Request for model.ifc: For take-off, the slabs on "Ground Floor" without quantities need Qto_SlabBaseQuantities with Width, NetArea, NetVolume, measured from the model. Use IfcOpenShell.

First a look at what the model holds.

```python
import ifcopenshell
import ifcopenshell.util.element
import ifcopenshell.util.unit

model = ifcopenshell.open("model.ifc")
print(model.schema)
for unit_type in ("LENGTHUNIT", "AREAUNIT", "VOLUMEUNIT"):
    print(unit_type, ifcopenshell.util.unit.calculate_unit_scale(model, unit_type))
storey = next(s for s in model.by_type("IfcBuildingStorey") if s.Name == "Ground Floor")
slabs = [e for e in ifcopenshell.util.element.get_decomposition(storey) if e.is_a("IfcSlab")]
for e in sorted(slabs, key=lambda e: e.id()):
    print(e.id(), e.is_a(), e.Name, list(ifcopenshell.util.element.get_psets(e, qtos_only=True)), sep=" | ")
```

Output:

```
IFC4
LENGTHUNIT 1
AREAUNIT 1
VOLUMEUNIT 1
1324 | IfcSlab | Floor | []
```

```python
import ifcopenshell
import ifcopenshell.api.pset
import ifcopenshell.geom
import ifcopenshell.util.element
import ifcopenshell.util.shape
import ifcopenshell.util.unit

model = ifcopenshell.open("model.ifc")
unit_scale = ifcopenshell.util.unit.calculate_unit_scale(model)
area_scale = ifcopenshell.util.unit.calculate_unit_scale(model, "AREAUNIT")
volume_scale = ifcopenshell.util.unit.calculate_unit_scale(model, "VOLUMEUNIT")
settings = ifcopenshell.geom.settings()

storey = next(s for s in model.by_type("IfcBuildingStorey") if s.Name == "Ground Floor")
slabs = [e for e in ifcopenshell.util.element.get_decomposition(storey) if e.is_a("IfcSlab")]

for e in sorted(slabs, key=lambda e: e.id()):
    if ifcopenshell.util.element.get_psets(e, qtos_only=True, should_inherit=False):
        continue
    # Geometry comes back in metres, in the element's own axes.
    shape = ifcopenshell.geom.create_shape(settings, e)
    values = {
        "Width": ifcopenshell.util.shape.get_z(shape.geometry) / unit_scale,
        "NetArea": ifcopenshell.util.shape.get_footprint_area(shape.geometry) / area_scale,
        "NetVolume": ifcopenshell.util.shape.get_volume(shape.geometry) / volume_scale,
    }
    qto = ifcopenshell.api.pset.add_qto(model, product=e, name="Qto_SlabBaseQuantities")
    ifcopenshell.api.pset.edit_qto(model, qto=qto, properties=values)
    print(e.id(), {k: round(v, 3) for k, v in values.items()})

model.write("model_v2.ifc")
```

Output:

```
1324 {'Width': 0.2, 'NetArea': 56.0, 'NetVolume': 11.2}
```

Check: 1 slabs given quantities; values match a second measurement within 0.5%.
